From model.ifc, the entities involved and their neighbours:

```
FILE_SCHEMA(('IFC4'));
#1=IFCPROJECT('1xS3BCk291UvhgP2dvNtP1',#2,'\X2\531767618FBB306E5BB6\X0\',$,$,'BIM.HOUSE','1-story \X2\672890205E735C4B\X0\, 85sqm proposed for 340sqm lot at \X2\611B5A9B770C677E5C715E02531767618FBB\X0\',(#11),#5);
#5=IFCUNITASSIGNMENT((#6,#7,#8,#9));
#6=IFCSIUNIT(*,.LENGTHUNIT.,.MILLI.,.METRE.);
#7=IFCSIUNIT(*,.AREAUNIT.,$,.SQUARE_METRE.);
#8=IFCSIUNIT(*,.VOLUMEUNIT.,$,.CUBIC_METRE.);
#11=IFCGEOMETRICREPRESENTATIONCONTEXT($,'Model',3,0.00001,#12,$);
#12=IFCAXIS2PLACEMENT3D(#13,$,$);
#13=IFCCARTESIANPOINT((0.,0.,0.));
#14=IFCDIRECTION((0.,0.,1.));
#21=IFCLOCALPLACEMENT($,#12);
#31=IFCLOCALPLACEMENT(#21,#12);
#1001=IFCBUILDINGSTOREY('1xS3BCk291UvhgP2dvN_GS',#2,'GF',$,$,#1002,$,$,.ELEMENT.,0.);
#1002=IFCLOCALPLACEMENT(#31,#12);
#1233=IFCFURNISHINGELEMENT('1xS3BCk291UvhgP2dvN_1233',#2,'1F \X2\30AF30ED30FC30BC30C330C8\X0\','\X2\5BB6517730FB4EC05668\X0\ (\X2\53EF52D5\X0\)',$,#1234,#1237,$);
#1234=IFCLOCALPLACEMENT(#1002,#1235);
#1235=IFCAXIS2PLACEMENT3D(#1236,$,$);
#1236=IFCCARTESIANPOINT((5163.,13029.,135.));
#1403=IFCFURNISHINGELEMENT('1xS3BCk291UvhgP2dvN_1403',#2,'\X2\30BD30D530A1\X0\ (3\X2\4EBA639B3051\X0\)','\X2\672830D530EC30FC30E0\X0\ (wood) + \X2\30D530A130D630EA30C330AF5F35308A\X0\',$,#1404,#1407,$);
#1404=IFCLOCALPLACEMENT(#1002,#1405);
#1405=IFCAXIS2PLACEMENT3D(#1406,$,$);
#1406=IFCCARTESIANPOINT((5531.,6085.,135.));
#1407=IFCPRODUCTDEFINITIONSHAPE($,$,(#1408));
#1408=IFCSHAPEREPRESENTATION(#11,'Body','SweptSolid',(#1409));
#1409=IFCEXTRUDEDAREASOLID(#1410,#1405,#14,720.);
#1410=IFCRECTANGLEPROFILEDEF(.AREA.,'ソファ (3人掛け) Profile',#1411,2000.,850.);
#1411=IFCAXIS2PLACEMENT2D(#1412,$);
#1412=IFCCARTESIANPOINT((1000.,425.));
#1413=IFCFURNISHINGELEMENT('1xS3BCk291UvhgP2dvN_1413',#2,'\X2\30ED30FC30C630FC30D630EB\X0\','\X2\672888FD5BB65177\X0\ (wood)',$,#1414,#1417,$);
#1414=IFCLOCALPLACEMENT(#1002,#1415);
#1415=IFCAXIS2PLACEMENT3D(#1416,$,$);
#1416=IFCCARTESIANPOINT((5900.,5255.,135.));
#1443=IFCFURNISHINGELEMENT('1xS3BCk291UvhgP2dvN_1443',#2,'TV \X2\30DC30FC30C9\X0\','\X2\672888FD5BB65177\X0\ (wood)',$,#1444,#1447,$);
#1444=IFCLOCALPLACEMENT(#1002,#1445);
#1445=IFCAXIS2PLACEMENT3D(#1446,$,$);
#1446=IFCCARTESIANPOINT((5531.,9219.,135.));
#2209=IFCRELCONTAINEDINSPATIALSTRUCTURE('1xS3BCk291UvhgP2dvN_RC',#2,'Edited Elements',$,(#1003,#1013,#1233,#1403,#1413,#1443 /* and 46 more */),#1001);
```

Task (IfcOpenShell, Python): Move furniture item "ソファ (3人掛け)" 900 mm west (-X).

```python
import ifcopenshell
import ifcopenshell.api.geometry
import ifcopenshell.util.placement
import ifcopenshell.util.unit

model = ifcopenshell.open("model.ifc")
unit_scale = ifcopenshell.util.unit.calculate_unit_scale(model)

item = model.by_guid("1xS3BCk291UvhgP2dvN_1403")
matrix = ifcopenshell.util.placement.get_local_placement(item.ObjectPlacement)
matrix[0, 3] -= 0.9 / unit_scale
ifcopenshell.api.geometry.edit_object_placement(model, product=item, matrix=matrix, is_si=False)

print(ifcopenshell.util.placement.get_local_placement(item.ObjectPlacement).round(3) + 0.0)

model.write("model_updated.ifc")
```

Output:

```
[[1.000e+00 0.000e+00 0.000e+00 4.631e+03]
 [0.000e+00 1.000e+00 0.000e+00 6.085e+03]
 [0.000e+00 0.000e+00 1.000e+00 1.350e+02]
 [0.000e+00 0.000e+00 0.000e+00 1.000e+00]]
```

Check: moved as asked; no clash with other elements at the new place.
